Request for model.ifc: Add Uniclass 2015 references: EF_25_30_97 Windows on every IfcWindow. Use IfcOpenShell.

First a look at what the model holds.

```python
import ifcopenshell

model = ifcopenshell.open("model.ifc")
print(model.schema)
print("classifications:", [c.Name for c in model.by_type("IfcClassification")])
for ifc_class in ("IfcDoor", "IfcRoof", "IfcStair", "IfcWall", "IfcWindow"):
    print(ifc_class, len(model.by_type(ifc_class)))
```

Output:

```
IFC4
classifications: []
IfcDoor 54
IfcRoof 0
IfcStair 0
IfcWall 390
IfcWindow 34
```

```python
import ifcopenshell
import ifcopenshell.api.classification

model = ifcopenshell.open("model.ifc")

system = ifcopenshell.api.classification.add_classification(model, classification="Uniclass 2015")

codes = {
    "IfcWindow": ("EF_25_30_97", "Windows"),
}
for ifc_class, (code, name) in codes.items():
    products = model.by_type(ifc_class)
    ifcopenshell.api.classification.add_reference(
        model, products=products, classification=system, identification=code, name=name
    )
    print(code, len(products))

model.write("model_edited.ifc")
```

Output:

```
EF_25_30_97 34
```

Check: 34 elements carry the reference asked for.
